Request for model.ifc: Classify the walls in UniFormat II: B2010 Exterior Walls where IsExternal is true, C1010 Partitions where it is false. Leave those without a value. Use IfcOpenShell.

First a look at what the model holds.

```python
import ifcopenshell
import ifcopenshell.util.element

model = ifcopenshell.open("model.ifc")
print(model.schema)
print("classifications:", [c.Name for c in model.by_type("IfcClassification")])
values = [ifcopenshell.util.element.get_pset(e, "Pset_WallCommon", "IsExternal") for e in model.by_type("IfcWall")]
for value in (True, False, None):
    print("IsExternal", value, values.count(value))
```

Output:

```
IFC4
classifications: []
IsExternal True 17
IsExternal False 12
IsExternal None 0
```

```python
import ifcopenshell
import ifcopenshell.api.classification
import ifcopenshell.util.element

model = ifcopenshell.open("model.ifc")

system = ifcopenshell.api.classification.add_classification(model, classification="UniFormat II")

walls = model.by_type("IfcWall")
external = {e: ifcopenshell.util.element.get_pset(e, "Pset_WallCommon", "IsExternal") for e in walls}
for flag, code, name in ((True, "B2010", "Exterior Walls"), (False, "C1010", "Partitions")):
    products = [e for e in walls if external[e] is flag]
    ifcopenshell.api.classification.add_reference(
        model, products=products, classification=system, identification=code, name=name
    )
    print(code, len(products))

model.write("model_updated.ifc")
```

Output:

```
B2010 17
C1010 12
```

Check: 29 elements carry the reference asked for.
